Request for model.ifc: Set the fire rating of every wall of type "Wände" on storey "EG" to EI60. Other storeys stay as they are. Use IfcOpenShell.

First a look at what the model holds.

```python
import ifcopenshell
import ifcopenshell.util.element

model = ifcopenshell.open("model.ifc")
print(model.schema)
storey = next(s for s in model.by_type("IfcBuildingStorey") if s.Name == "EG")
walls = [e for e in ifcopenshell.util.element.get_decomposition(storey) if e.is_a("IfcWall")]
seen = {}
for e in walls:
    element_type = ifcopenshell.util.element.get_type(e)
    key = (element_type.Name if element_type != e and element_type else None, ifcopenshell.util.element.get_pset(e, "Pset_WallCommon", "FireRating"))
    seen[key] = seen.get(key, 0) + 1
for (name, value), count in sorted(seen.items(), key=str):
    print(count, "x", name, "|", value)
```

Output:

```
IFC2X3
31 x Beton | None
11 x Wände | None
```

```python
import ifcopenshell
import ifcopenshell.api.pset
import ifcopenshell.util.element

model = ifcopenshell.open("model.ifc")

storey = next(s for s in model.by_type("IfcBuildingStorey") if s.Name == "EG")
walls = [e for e in ifcopenshell.util.element.get_decomposition(storey) if e.is_a("IfcWall")]

count = 0
for e in walls:
    element_type = ifcopenshell.util.element.get_type(e)
    if element_type in (None, e) or element_type.Name != "Wände":
        continue
    # add_pset returns the element's existing set when there is one.
    pset = ifcopenshell.api.pset.add_pset(model, product=e, name="Pset_WallCommon")
    ifcopenshell.api.pset.edit_pset(model, pset=pset, properties={"FireRating": "EI60"})
    count += 1

print(count, "walls updated")

model.write("model_rev.ifc")
```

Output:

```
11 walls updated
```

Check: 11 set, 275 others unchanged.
